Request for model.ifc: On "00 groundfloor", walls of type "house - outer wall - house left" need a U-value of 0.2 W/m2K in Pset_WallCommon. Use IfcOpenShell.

First a look at what the model holds.

```python
import ifcopenshell
import ifcopenshell.util.element

model = ifcopenshell.open("model.ifc")
print(model.schema)
storey = next(s for s in model.by_type("IfcBuildingStorey") if s.Name == "00 groundfloor")
walls = [e for e in ifcopenshell.util.element.get_decomposition(storey) if e.is_a("IfcWall")]
seen = {}
for e in walls:
    element_type = ifcopenshell.util.element.get_type(e)
    key = (element_type.Name if element_type != e and element_type else None, ifcopenshell.util.element.get_pset(e, "Pset_WallCommon", "ThermalTransmittance"))
    seen[key] = seen.get(key, 0) + 1
for (name, value), count in sorted(seen.items(), key=str):
    print(count, "x", name, "|", value)
```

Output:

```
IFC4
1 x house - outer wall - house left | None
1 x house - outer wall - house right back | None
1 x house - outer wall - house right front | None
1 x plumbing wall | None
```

```python
import ifcopenshell
import ifcopenshell.api.pset
import ifcopenshell.util.element

model = ifcopenshell.open("model.ifc")

storey = next(s for s in model.by_type("IfcBuildingStorey") if s.Name == "00 groundfloor")
walls = [e for e in ifcopenshell.util.element.get_decomposition(storey) if e.is_a("IfcWall")]

count = 0
for e in walls:
    element_type = ifcopenshell.util.element.get_type(e)
    if element_type in (None, e) or element_type.Name != "house - outer wall - house left":
        continue
    # add_pset returns the element's existing set when there is one.
    pset = ifcopenshell.api.pset.add_pset(model, product=e, name="Pset_WallCommon")
    ifcopenshell.api.pset.edit_pset(model, pset=pset, properties={"ThermalTransmittance": 0.2})
    count += 1

print(count, "walls updated")

model.write("model_edited.ifc")
```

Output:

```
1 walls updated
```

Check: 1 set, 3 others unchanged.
